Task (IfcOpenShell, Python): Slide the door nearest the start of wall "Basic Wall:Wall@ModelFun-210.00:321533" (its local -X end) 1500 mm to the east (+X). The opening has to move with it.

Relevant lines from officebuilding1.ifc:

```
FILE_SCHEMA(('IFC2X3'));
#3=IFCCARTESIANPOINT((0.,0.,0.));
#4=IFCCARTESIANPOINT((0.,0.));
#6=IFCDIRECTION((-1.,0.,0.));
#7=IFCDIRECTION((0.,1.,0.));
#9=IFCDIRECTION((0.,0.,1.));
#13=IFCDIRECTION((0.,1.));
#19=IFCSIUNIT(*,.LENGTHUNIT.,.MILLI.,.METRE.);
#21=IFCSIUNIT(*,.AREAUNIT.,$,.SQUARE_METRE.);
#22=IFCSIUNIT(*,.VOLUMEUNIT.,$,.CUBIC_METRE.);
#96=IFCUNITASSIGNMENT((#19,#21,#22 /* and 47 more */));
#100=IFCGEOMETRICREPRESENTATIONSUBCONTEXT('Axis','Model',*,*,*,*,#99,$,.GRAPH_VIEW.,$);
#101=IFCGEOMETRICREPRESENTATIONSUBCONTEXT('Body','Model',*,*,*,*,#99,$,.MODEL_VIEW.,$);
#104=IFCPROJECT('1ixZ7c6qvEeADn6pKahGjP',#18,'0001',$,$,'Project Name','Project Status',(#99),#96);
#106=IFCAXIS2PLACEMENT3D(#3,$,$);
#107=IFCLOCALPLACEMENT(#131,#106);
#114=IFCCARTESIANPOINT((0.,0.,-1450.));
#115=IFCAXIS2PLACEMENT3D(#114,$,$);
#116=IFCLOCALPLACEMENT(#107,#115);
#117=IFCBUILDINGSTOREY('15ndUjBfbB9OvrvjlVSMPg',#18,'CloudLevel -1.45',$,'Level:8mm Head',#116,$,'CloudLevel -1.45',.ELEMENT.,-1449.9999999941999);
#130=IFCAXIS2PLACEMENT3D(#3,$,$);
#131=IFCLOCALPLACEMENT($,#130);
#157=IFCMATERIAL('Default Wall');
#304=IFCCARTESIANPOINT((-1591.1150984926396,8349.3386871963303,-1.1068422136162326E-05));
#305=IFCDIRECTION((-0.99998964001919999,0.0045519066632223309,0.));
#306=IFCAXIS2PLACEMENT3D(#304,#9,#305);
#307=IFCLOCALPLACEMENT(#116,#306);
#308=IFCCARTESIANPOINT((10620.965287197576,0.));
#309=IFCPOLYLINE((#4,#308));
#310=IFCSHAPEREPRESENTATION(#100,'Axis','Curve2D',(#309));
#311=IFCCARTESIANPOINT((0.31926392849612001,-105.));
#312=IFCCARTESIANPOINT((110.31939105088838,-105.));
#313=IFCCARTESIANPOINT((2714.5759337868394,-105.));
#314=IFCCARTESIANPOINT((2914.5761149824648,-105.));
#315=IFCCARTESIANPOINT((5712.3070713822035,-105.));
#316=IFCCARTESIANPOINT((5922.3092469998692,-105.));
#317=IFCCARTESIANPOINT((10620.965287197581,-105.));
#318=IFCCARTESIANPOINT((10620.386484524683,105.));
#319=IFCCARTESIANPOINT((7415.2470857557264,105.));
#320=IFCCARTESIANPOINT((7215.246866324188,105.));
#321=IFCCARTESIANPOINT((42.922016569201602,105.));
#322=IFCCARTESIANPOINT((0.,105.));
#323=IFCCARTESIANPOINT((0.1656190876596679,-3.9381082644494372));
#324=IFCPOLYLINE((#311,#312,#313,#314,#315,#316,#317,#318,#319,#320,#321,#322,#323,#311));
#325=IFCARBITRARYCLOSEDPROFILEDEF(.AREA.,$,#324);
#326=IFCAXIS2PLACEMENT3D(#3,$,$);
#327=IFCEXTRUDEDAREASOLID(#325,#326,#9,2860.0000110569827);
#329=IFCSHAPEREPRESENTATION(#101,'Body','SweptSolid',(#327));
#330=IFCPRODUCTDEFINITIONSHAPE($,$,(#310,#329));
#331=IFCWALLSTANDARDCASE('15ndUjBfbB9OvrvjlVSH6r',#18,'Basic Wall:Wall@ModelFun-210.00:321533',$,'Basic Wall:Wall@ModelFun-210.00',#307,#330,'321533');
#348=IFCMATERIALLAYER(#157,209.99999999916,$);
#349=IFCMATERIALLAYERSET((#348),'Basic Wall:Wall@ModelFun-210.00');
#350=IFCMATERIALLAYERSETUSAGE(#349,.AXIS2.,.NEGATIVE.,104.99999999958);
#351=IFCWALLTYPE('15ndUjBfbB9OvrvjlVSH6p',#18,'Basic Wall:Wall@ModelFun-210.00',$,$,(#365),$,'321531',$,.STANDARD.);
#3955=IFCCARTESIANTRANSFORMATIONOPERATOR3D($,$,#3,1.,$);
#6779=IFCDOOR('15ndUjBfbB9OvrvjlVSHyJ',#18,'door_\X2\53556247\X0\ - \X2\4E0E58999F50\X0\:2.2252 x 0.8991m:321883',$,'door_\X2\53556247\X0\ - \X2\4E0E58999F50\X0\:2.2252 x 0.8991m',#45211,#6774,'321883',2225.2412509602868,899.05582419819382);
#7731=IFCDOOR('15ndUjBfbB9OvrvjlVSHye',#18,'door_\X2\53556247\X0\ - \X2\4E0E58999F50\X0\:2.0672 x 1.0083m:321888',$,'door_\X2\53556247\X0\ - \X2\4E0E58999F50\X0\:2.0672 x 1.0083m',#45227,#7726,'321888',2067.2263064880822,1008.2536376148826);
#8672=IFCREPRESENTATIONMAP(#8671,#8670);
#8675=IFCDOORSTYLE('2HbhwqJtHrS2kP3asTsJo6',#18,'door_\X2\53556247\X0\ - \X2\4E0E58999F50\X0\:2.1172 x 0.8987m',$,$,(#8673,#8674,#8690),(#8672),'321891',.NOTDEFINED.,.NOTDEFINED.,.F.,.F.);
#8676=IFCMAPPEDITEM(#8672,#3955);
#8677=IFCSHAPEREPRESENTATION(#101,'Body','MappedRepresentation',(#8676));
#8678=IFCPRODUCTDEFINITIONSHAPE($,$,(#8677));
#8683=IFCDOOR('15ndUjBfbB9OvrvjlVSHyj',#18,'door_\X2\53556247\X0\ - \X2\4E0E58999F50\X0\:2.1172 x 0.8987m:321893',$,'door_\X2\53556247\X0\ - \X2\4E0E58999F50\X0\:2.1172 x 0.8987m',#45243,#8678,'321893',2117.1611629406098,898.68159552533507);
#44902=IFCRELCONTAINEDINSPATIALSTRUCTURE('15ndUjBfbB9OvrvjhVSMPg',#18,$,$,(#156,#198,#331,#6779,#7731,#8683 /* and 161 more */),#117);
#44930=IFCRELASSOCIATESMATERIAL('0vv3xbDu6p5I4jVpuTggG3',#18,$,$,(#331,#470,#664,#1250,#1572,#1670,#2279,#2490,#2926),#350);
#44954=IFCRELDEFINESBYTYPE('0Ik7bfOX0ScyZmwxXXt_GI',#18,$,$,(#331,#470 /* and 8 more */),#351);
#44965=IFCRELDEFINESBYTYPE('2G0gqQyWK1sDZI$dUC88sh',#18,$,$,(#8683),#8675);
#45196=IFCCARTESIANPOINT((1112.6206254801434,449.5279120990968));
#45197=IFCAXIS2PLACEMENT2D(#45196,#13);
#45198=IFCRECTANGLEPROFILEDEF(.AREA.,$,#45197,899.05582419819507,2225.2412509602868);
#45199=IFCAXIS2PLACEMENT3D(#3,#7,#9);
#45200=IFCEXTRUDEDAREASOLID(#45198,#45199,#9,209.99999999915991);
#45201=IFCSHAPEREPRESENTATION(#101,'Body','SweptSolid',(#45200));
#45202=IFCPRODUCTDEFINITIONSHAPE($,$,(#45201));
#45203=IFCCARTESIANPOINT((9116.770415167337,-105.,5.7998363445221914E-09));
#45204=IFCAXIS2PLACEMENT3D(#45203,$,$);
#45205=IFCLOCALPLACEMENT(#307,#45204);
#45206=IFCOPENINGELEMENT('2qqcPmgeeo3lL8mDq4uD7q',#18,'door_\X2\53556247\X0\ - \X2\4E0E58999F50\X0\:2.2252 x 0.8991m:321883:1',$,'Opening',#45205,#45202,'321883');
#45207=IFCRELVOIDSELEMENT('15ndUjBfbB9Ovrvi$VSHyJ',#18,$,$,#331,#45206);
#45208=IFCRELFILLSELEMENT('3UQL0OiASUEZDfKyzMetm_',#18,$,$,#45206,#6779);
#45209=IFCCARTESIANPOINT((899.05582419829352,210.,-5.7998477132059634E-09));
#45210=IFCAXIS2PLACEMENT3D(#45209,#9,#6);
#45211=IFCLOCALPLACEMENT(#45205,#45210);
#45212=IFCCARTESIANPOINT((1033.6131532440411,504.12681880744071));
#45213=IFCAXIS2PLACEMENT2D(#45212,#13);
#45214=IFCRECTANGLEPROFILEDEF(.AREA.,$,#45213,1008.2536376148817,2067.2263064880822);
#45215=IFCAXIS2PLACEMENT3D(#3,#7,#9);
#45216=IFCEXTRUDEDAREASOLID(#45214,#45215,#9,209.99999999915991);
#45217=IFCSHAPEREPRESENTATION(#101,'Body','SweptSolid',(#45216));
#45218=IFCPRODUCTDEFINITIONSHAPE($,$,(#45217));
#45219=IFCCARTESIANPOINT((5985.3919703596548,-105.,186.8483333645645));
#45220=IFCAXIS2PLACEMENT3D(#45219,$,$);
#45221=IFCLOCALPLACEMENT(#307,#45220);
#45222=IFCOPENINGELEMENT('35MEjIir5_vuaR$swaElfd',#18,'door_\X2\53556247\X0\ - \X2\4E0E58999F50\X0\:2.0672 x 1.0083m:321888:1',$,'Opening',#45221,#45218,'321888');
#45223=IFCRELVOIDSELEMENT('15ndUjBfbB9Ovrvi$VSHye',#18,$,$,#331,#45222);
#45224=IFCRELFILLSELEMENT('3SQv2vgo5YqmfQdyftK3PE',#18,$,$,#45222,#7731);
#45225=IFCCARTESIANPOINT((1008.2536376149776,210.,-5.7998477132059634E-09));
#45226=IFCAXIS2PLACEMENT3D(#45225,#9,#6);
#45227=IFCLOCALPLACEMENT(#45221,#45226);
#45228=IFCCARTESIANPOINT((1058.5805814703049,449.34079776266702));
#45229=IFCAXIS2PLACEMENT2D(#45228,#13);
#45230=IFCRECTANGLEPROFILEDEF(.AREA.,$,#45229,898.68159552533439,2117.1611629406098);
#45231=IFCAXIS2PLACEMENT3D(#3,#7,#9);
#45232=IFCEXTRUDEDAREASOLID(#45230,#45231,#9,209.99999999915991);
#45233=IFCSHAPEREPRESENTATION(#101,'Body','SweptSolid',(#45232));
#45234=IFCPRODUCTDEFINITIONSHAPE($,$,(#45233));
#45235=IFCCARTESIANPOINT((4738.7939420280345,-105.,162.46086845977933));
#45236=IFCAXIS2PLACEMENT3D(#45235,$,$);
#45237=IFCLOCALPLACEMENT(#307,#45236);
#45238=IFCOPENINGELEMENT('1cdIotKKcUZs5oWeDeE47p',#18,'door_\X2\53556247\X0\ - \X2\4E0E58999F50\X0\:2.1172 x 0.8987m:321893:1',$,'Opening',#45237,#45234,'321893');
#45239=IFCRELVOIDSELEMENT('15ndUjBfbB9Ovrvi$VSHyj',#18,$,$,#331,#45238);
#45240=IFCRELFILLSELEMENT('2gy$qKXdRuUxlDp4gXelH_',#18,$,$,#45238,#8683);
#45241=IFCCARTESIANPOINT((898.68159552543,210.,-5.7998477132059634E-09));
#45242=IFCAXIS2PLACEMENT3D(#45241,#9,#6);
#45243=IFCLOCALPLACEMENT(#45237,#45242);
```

```python
import ifcopenshell
import ifcopenshell.api.geometry
import ifcopenshell.util.placement

model = ifcopenshell.open("officebuilding1.ifc")

door = model.by_guid("15ndUjBfbB9OvrvjlVSHyj")
opening = door.FillsVoids[0].RelatingOpeningElement
wall = opening.VoidsElements[0].RelatingBuildingElement

wall_matrix = ifcopenshell.util.placement.get_local_placement(wall.ObjectPlacement)
shift = wall_matrix[:3, 0] * -1500.0
before = ifcopenshell.util.placement.get_local_placement(door.ObjectPlacement)[:3, 3].copy()

# The door is placed relative to its opening, so it follows when the opening moves.
matrix = ifcopenshell.util.placement.get_local_placement(opening.ObjectPlacement)
matrix[:3, 3] += shift
ifcopenshell.api.geometry.edit_object_placement(
    model, product=opening, matrix=matrix, is_si=False, should_transform_children=True
)

after = ifcopenshell.util.placement.get_local_placement(door.ObjectPlacement)[:3, 3]
print("door moved by", (after - before).round(3) + 0.0)

model.write("officebuilding1-out.ifc")
```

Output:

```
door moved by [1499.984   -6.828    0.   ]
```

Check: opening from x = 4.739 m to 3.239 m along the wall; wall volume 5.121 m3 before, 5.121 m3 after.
